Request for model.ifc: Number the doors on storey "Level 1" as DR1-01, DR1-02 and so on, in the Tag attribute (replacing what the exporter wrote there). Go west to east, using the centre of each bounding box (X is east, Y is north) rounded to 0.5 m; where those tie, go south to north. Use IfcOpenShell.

First a look at what the model holds.

```python
import ifcopenshell
import ifcopenshell.util.element
import ifcopenshell.util.placement

model = ifcopenshell.open("model.ifc")
print(model.schema)
storey = next(s for s in model.by_type("IfcBuildingStorey") if s.Name == "Level 1")
doors = [e for e in ifcopenshell.util.element.get_decomposition(storey) if e.is_a("IfcDoor")]
for e in sorted(doors, key=lambda e: e.id()):
    origin = ifcopenshell.util.placement.get_local_placement(e.ObjectPlacement)[:3, 3]
    print(e.id(), e.Tag, e.Name, origin.round(2) + 0.0, sep=" | ")
```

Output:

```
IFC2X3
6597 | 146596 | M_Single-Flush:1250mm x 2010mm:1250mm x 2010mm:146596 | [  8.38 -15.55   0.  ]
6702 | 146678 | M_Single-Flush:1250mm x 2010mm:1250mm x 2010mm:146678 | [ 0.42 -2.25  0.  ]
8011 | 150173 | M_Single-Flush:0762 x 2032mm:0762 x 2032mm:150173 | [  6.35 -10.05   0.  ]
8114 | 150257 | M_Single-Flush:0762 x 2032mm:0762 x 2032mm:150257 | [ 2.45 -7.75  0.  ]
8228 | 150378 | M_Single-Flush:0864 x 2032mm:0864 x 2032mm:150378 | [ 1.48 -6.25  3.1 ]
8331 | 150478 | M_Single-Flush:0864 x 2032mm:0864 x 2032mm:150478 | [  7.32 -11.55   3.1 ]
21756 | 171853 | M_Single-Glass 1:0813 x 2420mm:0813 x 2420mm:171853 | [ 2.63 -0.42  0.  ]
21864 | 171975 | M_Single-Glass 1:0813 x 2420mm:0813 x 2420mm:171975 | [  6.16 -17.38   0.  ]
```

```python
import ifcopenshell
import ifcopenshell.geom
import ifcopenshell.util.element
import ifcopenshell.util.shape

model = ifcopenshell.open("model.ifc")
settings = ifcopenshell.geom.settings()
settings.set("use-world-coords", True)


def centre(element):
    shape = ifcopenshell.geom.create_shape(settings, element)
    return ifcopenshell.util.shape.get_bbox_centroid(shape.geometry)


storey = next(s for s in model.by_type("IfcBuildingStorey") if s.Name == "Level 1")
doors = [e for e in ifcopenshell.util.element.get_decomposition(storey) if e.is_a("IfcDoor")]

# Insertion points can sit at a corner or the storey origin, so sort by the geometry (in metres).
centres = {e: centre(e) for e in doors}
doors.sort(key=lambda e: (round(centres[e][0] / 0.5), centres[e][1]))

for i, e in enumerate(doors, start=1):
    number = f"DR1-{i:02d}"
    e.Tag = number
    print(e.id(), number)

model.write("model-out.ifc")
```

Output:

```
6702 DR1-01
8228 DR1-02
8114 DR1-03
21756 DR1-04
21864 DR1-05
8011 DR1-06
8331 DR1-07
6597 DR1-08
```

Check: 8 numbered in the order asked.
